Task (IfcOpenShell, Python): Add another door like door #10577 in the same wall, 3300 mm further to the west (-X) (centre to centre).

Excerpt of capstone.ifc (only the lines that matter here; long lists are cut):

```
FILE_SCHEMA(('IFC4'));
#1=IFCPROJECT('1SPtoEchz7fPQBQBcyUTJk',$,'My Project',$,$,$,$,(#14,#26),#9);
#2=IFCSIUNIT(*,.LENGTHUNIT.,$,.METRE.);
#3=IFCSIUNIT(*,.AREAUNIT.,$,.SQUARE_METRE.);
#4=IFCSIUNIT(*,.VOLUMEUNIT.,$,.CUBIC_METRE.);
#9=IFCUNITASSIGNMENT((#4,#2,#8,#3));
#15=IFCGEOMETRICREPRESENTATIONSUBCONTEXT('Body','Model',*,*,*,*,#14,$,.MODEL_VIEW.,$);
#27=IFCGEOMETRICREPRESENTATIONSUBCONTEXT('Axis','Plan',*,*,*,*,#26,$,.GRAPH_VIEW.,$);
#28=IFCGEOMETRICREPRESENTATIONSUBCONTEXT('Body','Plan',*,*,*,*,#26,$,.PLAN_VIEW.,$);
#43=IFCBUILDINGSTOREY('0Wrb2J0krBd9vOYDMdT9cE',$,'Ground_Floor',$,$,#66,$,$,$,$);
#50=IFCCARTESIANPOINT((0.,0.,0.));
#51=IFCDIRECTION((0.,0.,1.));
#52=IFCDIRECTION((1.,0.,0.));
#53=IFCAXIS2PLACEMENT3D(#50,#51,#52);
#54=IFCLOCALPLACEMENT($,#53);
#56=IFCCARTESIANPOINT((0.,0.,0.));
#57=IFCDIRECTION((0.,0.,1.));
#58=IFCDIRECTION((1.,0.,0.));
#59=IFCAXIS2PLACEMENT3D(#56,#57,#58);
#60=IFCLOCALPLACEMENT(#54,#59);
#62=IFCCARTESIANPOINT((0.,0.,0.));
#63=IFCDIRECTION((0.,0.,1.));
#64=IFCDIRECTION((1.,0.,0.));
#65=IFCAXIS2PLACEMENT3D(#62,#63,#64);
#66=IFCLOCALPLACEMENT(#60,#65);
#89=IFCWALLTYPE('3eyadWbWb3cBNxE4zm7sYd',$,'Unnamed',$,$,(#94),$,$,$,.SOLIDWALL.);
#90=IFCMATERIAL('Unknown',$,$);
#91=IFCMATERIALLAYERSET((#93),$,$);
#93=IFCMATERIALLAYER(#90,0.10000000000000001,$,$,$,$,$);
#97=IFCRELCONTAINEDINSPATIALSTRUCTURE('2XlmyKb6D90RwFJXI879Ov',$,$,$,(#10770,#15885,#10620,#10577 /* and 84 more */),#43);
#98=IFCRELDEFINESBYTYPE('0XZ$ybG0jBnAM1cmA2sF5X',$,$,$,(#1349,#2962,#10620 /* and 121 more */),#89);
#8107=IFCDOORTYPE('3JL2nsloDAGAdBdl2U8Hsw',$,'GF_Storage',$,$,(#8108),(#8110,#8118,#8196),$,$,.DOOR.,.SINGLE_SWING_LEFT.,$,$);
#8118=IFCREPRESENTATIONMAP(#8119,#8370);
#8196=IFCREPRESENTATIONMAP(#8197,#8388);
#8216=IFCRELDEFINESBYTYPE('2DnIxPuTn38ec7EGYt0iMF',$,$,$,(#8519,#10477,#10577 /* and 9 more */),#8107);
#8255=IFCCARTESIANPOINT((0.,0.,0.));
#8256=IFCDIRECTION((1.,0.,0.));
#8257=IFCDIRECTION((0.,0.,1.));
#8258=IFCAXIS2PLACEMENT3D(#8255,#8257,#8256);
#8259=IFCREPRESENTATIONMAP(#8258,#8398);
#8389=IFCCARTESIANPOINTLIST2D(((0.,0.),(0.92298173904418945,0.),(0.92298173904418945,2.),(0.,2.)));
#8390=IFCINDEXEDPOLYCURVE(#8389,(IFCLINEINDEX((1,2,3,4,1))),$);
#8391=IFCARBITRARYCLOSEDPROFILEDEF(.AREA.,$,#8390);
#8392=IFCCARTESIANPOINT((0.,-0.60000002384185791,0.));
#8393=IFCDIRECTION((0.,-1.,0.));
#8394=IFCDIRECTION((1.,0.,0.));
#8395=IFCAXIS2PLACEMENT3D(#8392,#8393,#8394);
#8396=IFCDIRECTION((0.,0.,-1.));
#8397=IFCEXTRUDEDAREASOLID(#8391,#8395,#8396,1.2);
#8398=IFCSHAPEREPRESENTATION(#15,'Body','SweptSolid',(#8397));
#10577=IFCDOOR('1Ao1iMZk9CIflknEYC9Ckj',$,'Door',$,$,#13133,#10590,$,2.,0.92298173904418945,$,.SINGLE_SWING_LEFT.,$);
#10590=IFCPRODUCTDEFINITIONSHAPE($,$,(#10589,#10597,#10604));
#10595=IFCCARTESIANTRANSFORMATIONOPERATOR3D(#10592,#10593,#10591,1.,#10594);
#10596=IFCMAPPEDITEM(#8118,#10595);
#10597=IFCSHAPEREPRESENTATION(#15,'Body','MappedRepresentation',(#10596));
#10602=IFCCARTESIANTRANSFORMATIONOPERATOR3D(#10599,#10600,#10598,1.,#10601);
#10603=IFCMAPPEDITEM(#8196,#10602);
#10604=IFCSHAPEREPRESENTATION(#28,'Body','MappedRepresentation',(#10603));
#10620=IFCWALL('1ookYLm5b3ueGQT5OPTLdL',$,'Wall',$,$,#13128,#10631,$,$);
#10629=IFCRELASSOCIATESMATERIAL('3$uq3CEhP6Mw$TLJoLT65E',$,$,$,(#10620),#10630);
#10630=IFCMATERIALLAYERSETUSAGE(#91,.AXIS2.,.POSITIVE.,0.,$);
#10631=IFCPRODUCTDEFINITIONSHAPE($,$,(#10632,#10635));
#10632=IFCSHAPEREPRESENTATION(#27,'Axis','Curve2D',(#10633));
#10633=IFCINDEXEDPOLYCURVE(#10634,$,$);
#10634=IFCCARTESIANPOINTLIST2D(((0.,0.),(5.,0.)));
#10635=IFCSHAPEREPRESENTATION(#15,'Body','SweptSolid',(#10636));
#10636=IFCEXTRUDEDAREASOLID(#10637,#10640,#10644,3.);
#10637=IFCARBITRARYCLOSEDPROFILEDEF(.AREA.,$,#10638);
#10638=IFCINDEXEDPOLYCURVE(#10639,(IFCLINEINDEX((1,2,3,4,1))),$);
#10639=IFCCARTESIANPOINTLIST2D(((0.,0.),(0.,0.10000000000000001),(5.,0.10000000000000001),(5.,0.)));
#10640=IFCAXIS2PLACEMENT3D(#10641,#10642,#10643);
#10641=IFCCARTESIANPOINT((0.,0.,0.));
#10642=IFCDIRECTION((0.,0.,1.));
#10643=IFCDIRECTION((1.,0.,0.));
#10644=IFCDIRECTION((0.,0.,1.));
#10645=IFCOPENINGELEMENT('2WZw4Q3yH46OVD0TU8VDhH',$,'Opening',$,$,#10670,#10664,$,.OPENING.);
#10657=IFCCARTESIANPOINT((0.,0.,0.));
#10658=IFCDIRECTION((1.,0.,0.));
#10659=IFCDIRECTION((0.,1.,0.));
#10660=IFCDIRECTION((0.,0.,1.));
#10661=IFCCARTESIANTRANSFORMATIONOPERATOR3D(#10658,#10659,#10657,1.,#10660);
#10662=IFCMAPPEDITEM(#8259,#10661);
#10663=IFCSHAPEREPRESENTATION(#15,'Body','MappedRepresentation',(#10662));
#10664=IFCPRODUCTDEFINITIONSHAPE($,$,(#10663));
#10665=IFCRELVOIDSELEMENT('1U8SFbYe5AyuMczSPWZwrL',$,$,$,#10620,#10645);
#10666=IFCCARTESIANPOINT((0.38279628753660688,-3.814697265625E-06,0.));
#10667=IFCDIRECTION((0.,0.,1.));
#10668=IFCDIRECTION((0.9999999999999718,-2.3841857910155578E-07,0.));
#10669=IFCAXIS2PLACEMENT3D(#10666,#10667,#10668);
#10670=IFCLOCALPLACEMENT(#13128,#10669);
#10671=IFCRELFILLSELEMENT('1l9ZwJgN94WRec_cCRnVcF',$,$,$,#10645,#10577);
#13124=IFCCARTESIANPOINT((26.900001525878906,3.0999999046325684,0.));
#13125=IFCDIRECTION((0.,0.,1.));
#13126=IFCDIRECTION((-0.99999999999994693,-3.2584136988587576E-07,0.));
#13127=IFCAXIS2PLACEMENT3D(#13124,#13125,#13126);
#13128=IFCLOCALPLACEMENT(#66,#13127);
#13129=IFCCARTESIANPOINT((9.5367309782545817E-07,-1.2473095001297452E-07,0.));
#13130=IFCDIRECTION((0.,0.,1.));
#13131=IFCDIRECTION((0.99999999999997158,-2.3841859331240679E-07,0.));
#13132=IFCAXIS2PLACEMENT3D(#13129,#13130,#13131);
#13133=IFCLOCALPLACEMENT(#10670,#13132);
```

```python
import ifcopenshell
import ifcopenshell.api.feature
import ifcopenshell.api.geometry
import ifcopenshell.api.root
import ifcopenshell.geom
import ifcopenshell.util.element
import ifcopenshell.util.placement
import ifcopenshell.util.shape
import ifcopenshell.util.unit

model = ifcopenshell.open("capstone.ifc")
unit_scale = ifcopenshell.util.unit.calculate_unit_scale(model)
settings = ifcopenshell.geom.settings()


def volume(element):
    """Net volume in cubic metres, openings subtracted."""
    shape = ifcopenshell.geom.create_shape(settings, element)
    return ifcopenshell.util.shape.get_volume(shape.geometry)


door = model.by_guid("1Ao1iMZk9CIflknEYC9Ckj")
opening = door.FillsVoids[0].RelatingOpeningElement
wall = opening.VoidsElements[0].RelatingBuildingElement
before = volume(wall)
shift = ifcopenshell.util.placement.get_local_placement(wall.ObjectPlacement)[:3, 0] * 3.3 / unit_scale

# copy_class copies the void relationship, type, container and properties, but no geometry.
new_opening = ifcopenshell.api.root.copy_class(model, product=opening)
new_opening.Representation = ifcopenshell.util.element.copy_deep(
    model, opening.Representation, exclude=["IfcGeometricRepresentationContext", "IfcRepresentationMap"]
)
new_door = ifcopenshell.api.root.copy_class(model, product=door)
new_door.Representation = ifcopenshell.util.element.copy_deep(
    model, door.Representation, exclude=["IfcGeometricRepresentationContext", "IfcRepresentationMap"]
)
ifcopenshell.api.feature.add_filling(model, opening=new_opening, element=new_door)

for old, new in ((opening, new_opening), (door, new_door)):
    matrix = ifcopenshell.util.placement.get_local_placement(old.ObjectPlacement)
    matrix[:3, 3] += shift
    ifcopenshell.api.geometry.edit_object_placement(model, product=new, matrix=matrix, is_si=False)

after = volume(wall)

print(f"wall volume {before:.3f} -> {after:.3f} m3")

model.write("capstone_rev.ifc")
```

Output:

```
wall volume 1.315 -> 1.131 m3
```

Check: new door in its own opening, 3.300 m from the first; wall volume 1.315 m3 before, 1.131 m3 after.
